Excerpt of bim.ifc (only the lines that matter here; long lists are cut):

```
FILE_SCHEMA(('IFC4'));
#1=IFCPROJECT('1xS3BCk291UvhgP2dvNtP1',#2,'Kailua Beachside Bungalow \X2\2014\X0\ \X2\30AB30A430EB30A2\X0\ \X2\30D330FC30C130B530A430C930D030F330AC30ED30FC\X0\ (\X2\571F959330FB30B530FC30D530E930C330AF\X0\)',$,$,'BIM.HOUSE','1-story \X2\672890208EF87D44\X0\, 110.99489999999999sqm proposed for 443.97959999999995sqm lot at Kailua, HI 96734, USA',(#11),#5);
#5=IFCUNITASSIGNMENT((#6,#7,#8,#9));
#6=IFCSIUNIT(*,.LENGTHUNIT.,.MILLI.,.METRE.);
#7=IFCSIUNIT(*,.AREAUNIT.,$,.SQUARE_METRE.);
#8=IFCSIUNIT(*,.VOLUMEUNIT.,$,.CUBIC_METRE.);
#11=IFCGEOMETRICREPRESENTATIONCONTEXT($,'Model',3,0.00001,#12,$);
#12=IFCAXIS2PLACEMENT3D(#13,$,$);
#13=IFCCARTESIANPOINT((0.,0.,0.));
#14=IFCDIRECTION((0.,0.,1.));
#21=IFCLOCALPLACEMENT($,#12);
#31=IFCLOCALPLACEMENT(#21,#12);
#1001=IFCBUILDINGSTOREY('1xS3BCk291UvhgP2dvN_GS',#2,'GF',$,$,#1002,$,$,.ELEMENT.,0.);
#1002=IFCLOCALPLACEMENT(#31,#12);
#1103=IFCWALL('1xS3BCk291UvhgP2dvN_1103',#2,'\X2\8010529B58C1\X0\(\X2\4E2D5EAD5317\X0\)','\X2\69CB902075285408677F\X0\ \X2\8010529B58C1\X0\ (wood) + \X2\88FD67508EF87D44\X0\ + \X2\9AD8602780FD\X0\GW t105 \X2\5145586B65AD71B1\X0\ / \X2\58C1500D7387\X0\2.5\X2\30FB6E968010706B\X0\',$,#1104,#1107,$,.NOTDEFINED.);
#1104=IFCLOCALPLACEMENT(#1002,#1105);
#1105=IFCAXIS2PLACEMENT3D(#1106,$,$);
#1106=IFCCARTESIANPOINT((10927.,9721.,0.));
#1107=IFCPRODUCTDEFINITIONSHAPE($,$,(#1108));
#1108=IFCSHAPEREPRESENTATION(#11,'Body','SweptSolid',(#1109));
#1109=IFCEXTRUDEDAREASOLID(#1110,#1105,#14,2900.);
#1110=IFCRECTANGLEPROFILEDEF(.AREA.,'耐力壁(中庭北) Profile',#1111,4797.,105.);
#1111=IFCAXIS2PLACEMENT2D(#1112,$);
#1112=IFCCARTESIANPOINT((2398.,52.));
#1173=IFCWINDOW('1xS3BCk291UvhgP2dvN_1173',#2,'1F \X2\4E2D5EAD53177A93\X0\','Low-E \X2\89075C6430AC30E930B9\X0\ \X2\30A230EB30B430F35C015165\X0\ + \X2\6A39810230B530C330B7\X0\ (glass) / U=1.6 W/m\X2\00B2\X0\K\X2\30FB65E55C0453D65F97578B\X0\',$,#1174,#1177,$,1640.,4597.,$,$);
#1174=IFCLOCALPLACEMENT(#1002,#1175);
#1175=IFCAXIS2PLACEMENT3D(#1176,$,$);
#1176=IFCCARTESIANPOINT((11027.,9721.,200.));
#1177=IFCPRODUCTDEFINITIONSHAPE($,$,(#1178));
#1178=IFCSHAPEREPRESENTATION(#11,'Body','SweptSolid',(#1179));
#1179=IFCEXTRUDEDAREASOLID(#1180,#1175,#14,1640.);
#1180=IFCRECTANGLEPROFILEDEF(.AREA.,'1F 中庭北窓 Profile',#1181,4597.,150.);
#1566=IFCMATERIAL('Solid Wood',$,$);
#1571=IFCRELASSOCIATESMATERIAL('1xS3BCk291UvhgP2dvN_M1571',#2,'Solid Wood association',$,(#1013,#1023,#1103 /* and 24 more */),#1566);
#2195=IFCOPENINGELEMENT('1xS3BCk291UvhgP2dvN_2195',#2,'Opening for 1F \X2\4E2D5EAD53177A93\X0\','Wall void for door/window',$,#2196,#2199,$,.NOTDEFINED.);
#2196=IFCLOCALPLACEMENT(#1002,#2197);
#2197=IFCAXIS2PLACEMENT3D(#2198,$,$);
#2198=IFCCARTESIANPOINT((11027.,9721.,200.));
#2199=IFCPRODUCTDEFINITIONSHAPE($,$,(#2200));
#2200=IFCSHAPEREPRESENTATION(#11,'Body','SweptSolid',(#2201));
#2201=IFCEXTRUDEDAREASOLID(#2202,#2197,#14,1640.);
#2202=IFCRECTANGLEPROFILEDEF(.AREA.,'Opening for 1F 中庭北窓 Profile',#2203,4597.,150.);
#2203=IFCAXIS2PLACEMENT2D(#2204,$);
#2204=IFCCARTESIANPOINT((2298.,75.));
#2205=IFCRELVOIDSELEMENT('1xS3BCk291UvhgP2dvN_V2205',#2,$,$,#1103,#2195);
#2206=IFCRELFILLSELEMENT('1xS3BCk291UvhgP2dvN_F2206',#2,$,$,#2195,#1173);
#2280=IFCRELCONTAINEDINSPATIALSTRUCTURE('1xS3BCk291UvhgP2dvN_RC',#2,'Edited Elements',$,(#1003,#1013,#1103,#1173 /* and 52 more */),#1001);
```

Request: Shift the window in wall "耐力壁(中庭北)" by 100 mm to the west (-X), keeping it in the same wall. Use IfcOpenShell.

```python
import ifcopenshell
import ifcopenshell.api.geometry
import ifcopenshell.util.placement

model = ifcopenshell.open("bim.ifc")

window = model.by_guid("1xS3BCk291UvhgP2dvN_1173")
opening = window.FillsVoids[0].RelatingOpeningElement
wall = opening.VoidsElements[0].RelatingBuildingElement

wall_matrix = ifcopenshell.util.placement.get_local_placement(wall.ObjectPlacement)
shift = wall_matrix[:3, 0] * -100.0
before = ifcopenshell.util.placement.get_local_placement(window.ObjectPlacement)[:3, 3].copy()

# The window is not placed relative to its opening, so move both.
for product in (opening, window):
    matrix = ifcopenshell.util.placement.get_local_placement(product.ObjectPlacement)
    matrix[:3, 3] += shift
    ifcopenshell.api.geometry.edit_object_placement(model, product=product, matrix=matrix, is_si=False)

after = ifcopenshell.util.placement.get_local_placement(window.ObjectPlacement)[:3, 3]
print("window moved by", (after - before).round(3) + 0.0)

model.write("bim_edited.ifc")
```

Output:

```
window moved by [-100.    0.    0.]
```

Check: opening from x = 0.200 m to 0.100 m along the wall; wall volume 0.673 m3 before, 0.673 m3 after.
